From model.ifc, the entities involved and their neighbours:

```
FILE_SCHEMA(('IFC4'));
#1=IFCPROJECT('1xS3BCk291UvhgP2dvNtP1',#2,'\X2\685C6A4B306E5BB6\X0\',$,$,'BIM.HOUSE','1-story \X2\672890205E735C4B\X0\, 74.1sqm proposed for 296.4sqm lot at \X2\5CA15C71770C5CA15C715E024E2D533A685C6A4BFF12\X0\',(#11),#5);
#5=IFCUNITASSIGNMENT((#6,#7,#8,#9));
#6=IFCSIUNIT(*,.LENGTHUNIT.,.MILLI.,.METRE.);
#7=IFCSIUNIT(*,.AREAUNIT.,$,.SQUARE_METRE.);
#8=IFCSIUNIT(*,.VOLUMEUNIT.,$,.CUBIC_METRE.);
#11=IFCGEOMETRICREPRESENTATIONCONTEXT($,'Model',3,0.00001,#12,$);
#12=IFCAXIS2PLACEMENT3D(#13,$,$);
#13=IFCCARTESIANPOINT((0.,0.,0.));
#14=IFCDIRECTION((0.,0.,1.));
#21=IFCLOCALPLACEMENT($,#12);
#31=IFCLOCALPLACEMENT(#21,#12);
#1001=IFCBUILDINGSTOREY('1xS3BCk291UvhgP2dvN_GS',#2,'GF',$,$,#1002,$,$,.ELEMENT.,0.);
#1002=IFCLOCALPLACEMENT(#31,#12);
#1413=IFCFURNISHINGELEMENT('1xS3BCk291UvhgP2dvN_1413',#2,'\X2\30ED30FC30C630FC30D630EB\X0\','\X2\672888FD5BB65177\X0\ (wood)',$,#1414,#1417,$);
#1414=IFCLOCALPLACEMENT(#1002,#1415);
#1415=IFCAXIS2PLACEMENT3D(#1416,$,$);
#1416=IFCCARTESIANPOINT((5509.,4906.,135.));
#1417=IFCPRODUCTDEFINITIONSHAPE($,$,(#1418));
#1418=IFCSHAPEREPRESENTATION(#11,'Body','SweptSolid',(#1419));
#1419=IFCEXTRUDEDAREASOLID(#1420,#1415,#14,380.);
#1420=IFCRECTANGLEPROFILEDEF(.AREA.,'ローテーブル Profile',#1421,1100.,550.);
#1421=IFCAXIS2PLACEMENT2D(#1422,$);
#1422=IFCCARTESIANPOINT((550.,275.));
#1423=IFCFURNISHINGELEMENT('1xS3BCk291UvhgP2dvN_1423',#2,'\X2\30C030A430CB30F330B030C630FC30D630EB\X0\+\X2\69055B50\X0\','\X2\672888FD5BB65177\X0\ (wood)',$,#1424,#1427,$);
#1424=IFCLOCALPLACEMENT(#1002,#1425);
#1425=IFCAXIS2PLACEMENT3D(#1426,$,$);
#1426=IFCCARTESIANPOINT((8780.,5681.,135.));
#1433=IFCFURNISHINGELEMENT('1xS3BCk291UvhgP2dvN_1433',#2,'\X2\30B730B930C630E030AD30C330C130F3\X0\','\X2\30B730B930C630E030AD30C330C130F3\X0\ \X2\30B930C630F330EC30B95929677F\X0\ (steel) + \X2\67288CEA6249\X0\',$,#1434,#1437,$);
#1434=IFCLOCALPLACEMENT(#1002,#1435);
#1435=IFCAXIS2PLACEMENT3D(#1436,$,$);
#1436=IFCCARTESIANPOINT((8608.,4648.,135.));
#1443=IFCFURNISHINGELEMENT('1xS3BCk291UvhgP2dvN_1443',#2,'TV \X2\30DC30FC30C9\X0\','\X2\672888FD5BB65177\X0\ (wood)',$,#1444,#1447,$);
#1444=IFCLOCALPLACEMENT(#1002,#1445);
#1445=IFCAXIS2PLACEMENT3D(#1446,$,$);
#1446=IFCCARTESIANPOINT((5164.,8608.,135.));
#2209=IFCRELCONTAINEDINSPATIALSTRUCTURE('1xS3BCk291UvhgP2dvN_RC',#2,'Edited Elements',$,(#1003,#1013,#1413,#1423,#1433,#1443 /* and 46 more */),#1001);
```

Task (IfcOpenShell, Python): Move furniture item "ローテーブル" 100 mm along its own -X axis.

```python
import ifcopenshell
import ifcopenshell.api.geometry
import ifcopenshell.util.placement
import ifcopenshell.util.unit

model = ifcopenshell.open("model.ifc")
unit_scale = ifcopenshell.util.unit.calculate_unit_scale(model)

item = model.by_guid("1xS3BCk291UvhgP2dvN_1413")
matrix = ifcopenshell.util.placement.get_local_placement(item.ObjectPlacement)
matrix[:3, 3] -= matrix[:3, 0] * 0.1 / unit_scale
ifcopenshell.api.geometry.edit_object_placement(model, product=item, matrix=matrix, is_si=False)

print(ifcopenshell.util.placement.get_local_placement(item.ObjectPlacement).round(3) + 0.0)

model.write("model_rev.ifc")
```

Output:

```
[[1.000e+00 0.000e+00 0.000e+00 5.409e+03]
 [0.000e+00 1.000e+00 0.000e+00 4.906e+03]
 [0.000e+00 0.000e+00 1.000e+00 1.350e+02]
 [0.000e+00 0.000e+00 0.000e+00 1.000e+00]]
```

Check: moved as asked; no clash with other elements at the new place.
